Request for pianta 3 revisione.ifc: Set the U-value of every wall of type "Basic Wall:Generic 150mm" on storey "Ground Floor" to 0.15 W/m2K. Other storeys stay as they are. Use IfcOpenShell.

First a look at what the model holds.

```python
import ifcopenshell
import ifcopenshell.util.element

model = ifcopenshell.open("pianta 3 revisione.ifc")
print(model.schema)
storey = next(s for s in model.by_type("IfcBuildingStorey") if s.Name == "Ground Floor")
walls = [e for e in ifcopenshell.util.element.get_decomposition(storey) if e.is_a("IfcWall")]
seen = {}
for e in walls:
    element_type = ifcopenshell.util.element.get_type(e)
    key = (element_type.Name if element_type != e and element_type else None, ifcopenshell.util.element.get_pset(e, "Pset_WallCommon", "ThermalTransmittance"))
    seen[key] = seen.get(key, 0) + 1
for (name, value), count in sorted(seen.items(), key=str):
    print(count, "x", name, "|", value)
```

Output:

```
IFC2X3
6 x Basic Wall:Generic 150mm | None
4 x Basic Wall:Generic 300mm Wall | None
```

```python
import ifcopenshell
import ifcopenshell.api.pset
import ifcopenshell.util.element

model = ifcopenshell.open("pianta 3 revisione.ifc")

storey = next(s for s in model.by_type("IfcBuildingStorey") if s.Name == "Ground Floor")
walls = [e for e in ifcopenshell.util.element.get_decomposition(storey) if e.is_a("IfcWall")]

count = 0
for e in walls:
    element_type = ifcopenshell.util.element.get_type(e)
    if element_type in (None, e) or element_type.Name != "Basic Wall:Generic 150mm":
        continue
    # add_pset returns the element's existing set when there is one.
    pset = ifcopenshell.api.pset.add_pset(model, product=e, name="Pset_WallCommon")
    ifcopenshell.api.pset.edit_pset(model, pset=pset, properties={"ThermalTransmittance": 0.15})
    count += 1

print(count, "walls updated")

model.write("pianta 3 revisione_rev.ifc")
```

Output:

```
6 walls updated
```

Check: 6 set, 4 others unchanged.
